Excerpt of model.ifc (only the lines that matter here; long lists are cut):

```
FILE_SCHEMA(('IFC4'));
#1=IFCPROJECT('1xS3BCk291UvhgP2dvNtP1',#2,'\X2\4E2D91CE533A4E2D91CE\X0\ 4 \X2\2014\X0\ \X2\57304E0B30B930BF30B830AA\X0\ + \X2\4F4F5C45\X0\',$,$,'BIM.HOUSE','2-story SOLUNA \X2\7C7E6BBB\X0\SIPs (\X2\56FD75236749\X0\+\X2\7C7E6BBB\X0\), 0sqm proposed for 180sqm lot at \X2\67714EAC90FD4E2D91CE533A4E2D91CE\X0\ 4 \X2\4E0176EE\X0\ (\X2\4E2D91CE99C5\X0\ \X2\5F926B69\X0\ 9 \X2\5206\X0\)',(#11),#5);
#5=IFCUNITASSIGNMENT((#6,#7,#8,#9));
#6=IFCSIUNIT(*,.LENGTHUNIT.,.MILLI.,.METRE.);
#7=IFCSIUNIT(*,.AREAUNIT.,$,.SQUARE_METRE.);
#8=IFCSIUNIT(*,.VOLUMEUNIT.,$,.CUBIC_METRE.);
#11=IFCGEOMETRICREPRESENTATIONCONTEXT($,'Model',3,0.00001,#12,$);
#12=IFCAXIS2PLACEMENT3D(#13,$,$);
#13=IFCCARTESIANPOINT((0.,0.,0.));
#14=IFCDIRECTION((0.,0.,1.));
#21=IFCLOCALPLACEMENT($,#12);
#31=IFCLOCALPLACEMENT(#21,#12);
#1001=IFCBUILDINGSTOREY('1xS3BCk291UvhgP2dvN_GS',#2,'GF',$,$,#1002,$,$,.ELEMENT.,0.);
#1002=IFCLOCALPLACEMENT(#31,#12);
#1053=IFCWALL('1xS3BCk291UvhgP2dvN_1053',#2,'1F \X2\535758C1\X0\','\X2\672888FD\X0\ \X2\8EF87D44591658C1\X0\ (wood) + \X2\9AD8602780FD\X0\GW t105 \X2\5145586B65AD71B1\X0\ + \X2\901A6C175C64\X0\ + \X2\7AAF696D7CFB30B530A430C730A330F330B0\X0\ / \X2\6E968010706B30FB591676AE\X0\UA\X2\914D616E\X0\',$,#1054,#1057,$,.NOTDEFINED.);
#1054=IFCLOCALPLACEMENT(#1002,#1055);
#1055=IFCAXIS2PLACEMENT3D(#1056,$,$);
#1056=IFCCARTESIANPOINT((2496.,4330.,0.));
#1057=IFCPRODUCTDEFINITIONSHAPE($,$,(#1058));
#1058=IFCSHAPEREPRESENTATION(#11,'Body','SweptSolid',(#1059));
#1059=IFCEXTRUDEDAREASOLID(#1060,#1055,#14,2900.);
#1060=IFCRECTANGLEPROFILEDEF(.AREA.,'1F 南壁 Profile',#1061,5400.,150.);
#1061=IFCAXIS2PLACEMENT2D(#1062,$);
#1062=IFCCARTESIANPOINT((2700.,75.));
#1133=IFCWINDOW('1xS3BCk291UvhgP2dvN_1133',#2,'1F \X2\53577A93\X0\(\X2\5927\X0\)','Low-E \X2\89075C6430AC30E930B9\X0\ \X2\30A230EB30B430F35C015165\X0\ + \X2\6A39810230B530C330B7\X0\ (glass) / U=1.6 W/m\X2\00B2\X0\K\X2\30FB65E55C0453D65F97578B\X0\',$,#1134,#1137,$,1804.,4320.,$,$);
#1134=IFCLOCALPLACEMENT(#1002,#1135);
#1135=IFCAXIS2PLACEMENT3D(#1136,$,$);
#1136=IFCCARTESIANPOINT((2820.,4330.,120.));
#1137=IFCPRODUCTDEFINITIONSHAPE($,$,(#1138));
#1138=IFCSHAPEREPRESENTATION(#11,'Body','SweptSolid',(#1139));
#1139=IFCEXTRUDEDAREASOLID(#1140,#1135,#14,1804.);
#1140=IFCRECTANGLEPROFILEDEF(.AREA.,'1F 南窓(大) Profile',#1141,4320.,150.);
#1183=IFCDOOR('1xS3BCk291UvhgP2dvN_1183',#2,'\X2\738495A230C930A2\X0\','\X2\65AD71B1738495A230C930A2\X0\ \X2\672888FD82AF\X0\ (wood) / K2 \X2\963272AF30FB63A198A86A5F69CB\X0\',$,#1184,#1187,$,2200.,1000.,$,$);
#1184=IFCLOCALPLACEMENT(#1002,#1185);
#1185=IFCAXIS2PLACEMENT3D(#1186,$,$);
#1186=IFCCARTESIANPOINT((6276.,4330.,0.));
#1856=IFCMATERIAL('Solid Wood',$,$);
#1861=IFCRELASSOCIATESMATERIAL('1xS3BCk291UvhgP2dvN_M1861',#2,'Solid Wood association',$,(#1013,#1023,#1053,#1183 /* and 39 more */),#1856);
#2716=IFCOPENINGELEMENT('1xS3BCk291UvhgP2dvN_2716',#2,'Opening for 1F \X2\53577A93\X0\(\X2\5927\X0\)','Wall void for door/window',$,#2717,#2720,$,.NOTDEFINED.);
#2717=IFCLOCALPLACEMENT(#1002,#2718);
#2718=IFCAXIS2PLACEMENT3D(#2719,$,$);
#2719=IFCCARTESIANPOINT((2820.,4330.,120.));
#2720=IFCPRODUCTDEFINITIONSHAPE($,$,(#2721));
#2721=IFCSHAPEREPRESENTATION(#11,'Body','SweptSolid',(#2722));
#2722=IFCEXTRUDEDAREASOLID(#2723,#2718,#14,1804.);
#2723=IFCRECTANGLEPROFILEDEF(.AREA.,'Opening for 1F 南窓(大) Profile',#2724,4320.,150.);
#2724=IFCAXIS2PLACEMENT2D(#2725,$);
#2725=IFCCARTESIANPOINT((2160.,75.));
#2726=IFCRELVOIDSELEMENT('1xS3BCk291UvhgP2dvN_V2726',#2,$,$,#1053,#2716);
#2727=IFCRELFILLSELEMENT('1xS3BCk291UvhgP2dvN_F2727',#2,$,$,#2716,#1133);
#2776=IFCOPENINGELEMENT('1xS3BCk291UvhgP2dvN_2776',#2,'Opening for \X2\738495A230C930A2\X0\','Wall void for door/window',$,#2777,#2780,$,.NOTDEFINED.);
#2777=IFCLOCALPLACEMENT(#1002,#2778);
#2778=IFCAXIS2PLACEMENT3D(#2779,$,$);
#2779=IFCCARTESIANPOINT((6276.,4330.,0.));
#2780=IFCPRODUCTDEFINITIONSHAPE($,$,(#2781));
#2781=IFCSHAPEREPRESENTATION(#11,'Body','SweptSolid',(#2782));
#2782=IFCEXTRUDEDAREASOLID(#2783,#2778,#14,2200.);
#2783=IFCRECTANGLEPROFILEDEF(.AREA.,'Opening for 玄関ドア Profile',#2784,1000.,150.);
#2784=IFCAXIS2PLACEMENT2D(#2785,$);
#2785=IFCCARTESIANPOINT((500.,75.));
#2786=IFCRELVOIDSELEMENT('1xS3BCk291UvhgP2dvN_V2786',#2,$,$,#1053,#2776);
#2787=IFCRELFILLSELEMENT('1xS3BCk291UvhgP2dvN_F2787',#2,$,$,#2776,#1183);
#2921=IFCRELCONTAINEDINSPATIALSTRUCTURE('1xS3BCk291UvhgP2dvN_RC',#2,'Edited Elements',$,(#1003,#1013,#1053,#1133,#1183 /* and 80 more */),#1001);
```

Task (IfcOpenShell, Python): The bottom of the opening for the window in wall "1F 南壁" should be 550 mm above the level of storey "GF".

```python
import numpy as np
import ifcopenshell
import ifcopenshell.api.geometry
import ifcopenshell.geom
import ifcopenshell.util.element
import ifcopenshell.util.placement
import ifcopenshell.util.shape
import ifcopenshell.util.unit

model = ifcopenshell.open("model.ifc")
unit_scale = ifcopenshell.util.unit.calculate_unit_scale(model)

window = model.by_id(1133)
opening = window.FillsVoids[0].RelatingOpeningElement
storey = ifcopenshell.util.element.get_container(window, ifc_class="IfcBuildingStorey")
level = ifcopenshell.util.placement.get_local_placement(storey.ObjectPlacement)[2, 3]

# The opening's origin need not be at the sill, so measure its lowest point.
shape = ifcopenshell.geom.create_shape(ifcopenshell.geom.settings(), opening)
bottom = ifcopenshell.util.shape.get_shape_bottom_elevation(shape, shape.geometry) / unit_scale
dz = level + 0.55 / unit_scale - bottom

shift = np.array([0.0, 0.0, dz])
# The window is not placed relative to its opening, so move both.
for product in (opening, window):
    matrix = ifcopenshell.util.placement.get_local_placement(product.ObjectPlacement)
    matrix[:3, 3] += shift
    ifcopenshell.api.geometry.edit_object_placement(model, product=product, matrix=matrix, is_si=False)

print(f"moved by {dz * unit_scale:+.3f} m")

model.write("model-out.ifc")
```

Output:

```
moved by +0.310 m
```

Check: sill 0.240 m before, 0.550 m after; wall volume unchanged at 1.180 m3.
